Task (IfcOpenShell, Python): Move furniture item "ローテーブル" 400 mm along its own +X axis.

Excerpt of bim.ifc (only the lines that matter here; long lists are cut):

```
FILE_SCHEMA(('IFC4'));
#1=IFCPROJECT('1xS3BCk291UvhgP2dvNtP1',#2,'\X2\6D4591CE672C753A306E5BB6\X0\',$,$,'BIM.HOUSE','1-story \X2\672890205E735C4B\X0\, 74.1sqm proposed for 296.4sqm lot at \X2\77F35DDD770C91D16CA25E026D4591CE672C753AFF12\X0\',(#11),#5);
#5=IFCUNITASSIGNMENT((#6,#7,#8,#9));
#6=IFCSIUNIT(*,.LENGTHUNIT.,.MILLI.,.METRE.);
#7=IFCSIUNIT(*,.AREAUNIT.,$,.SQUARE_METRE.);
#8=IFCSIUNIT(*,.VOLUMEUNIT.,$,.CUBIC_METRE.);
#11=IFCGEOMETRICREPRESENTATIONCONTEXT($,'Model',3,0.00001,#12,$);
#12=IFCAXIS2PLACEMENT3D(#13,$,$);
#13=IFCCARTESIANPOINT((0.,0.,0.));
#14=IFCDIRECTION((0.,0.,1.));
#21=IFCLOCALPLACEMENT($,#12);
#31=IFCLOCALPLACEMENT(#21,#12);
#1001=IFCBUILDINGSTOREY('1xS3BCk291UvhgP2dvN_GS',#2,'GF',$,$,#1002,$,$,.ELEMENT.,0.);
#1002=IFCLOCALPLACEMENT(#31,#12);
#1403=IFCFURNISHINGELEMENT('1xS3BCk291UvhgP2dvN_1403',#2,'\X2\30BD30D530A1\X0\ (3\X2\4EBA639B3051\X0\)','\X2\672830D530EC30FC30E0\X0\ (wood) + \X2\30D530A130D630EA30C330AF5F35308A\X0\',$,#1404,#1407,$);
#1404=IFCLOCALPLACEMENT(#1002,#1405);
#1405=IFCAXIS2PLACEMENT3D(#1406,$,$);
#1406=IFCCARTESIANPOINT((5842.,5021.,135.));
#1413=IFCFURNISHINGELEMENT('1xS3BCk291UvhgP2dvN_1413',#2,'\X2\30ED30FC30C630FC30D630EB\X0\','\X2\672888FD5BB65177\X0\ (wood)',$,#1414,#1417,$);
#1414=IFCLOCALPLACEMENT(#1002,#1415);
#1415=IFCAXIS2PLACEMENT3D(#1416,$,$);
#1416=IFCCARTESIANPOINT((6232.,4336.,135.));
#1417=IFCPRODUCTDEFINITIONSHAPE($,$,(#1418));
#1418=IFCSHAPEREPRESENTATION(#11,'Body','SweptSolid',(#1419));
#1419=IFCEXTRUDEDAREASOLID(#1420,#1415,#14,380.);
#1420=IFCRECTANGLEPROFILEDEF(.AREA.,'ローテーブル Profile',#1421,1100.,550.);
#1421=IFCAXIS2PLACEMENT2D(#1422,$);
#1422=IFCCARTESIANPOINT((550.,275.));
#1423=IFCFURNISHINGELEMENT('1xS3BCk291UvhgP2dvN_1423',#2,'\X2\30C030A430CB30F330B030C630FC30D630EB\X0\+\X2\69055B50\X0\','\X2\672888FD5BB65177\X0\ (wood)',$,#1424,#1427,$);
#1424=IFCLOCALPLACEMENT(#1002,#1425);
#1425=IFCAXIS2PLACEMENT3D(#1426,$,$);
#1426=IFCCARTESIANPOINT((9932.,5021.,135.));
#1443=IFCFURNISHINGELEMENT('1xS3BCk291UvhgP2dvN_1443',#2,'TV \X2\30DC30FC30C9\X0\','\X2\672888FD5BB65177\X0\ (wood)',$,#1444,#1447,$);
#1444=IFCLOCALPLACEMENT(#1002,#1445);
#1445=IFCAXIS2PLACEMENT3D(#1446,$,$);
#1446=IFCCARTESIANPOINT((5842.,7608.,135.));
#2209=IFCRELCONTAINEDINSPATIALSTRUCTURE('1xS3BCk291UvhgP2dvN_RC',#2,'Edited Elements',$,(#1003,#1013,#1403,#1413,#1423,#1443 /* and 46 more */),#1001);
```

```python
import ifcopenshell
import ifcopenshell.api.geometry
import ifcopenshell.util.placement
import ifcopenshell.util.unit

model = ifcopenshell.open("bim.ifc")
unit_scale = ifcopenshell.util.unit.calculate_unit_scale(model)

item = model.by_id(1413)
matrix = ifcopenshell.util.placement.get_local_placement(item.ObjectPlacement)
matrix[:3, 3] += matrix[:3, 0] * 0.4 / unit_scale
ifcopenshell.api.geometry.edit_object_placement(model, product=item, matrix=matrix, is_si=False)

print(ifcopenshell.util.placement.get_local_placement(item.ObjectPlacement).round(3) + 0.0)

model.write("bim_edited.ifc")
```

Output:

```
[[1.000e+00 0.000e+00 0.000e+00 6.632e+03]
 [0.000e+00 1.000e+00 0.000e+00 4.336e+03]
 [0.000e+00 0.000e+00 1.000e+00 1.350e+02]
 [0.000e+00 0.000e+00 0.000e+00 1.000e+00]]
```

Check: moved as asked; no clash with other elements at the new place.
